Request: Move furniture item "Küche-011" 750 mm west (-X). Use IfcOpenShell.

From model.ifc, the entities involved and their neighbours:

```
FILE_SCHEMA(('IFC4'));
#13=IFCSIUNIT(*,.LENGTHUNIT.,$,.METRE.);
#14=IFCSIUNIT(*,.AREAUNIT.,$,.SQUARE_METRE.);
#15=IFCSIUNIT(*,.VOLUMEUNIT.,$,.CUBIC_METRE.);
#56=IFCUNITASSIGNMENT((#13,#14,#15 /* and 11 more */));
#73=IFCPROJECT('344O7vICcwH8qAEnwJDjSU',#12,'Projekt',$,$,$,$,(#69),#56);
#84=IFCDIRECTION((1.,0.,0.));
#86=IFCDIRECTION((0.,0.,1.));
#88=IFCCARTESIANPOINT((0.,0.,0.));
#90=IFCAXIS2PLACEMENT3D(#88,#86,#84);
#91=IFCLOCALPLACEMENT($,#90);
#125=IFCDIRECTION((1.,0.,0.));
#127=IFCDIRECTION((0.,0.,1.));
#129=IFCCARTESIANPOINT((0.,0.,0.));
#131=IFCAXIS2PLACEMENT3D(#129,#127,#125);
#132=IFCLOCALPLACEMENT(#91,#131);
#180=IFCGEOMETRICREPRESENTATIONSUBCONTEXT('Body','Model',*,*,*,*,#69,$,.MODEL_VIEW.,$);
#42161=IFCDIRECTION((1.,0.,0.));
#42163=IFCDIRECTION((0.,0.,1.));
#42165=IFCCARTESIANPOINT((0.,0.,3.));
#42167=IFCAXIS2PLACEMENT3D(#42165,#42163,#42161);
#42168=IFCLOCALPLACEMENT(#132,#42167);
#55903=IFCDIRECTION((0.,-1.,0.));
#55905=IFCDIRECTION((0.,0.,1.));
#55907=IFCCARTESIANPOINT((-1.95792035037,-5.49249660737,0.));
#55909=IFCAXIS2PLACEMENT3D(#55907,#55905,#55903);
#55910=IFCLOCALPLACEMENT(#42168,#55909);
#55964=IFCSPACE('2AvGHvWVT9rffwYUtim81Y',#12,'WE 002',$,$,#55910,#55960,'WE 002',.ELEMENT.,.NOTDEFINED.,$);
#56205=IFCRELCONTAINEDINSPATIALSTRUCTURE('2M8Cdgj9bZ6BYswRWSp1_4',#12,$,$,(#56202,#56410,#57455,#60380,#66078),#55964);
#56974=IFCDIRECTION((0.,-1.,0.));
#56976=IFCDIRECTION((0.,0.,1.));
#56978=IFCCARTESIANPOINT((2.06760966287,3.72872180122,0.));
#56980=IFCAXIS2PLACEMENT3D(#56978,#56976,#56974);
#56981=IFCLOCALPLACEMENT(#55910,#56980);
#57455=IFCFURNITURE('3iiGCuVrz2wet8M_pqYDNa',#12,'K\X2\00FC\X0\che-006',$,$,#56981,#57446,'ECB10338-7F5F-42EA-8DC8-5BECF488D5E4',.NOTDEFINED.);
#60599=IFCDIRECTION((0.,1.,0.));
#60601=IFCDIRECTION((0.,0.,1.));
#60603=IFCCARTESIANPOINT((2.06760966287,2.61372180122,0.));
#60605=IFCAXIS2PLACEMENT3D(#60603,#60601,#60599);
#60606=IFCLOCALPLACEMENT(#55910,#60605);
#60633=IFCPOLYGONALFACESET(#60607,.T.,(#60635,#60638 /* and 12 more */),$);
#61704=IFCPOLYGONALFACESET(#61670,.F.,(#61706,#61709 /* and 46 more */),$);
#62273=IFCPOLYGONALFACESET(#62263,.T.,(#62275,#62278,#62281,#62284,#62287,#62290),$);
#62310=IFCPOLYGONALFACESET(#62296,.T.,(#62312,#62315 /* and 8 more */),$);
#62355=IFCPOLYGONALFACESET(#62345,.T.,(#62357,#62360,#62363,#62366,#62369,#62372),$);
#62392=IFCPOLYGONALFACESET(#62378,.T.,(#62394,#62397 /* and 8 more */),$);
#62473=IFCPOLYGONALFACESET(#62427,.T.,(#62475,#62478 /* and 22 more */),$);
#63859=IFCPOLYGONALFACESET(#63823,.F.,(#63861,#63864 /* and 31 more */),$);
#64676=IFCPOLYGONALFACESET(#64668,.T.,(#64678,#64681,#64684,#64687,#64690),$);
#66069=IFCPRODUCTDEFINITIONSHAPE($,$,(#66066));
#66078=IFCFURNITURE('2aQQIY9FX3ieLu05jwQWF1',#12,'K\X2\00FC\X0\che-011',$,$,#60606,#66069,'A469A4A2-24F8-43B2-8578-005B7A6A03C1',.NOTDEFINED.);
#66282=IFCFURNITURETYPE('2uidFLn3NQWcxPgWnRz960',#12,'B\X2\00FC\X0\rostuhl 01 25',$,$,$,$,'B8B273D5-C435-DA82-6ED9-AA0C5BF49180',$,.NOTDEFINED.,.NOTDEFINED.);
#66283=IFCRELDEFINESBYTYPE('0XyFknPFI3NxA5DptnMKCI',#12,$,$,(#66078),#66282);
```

```python
import ifcopenshell
import ifcopenshell.api.geometry
import ifcopenshell.util.placement
import ifcopenshell.util.unit

model = ifcopenshell.open("model.ifc")
unit_scale = ifcopenshell.util.unit.calculate_unit_scale(model)

item = model.by_id(66078)
matrix = ifcopenshell.util.placement.get_local_placement(item.ObjectPlacement)
matrix[0, 3] -= 0.75 / unit_scale
ifcopenshell.api.geometry.edit_object_placement(model, product=item, matrix=matrix, is_si=False)

print(ifcopenshell.util.placement.get_local_placement(item.ObjectPlacement).round(3) + 0.0)

model.write("model_v2.ifc")
```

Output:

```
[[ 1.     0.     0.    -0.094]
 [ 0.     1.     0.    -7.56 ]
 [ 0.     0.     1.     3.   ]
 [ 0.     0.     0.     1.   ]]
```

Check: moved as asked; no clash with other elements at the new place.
